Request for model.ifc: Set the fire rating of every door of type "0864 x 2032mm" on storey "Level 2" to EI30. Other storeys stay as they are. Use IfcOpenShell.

First a look at what the model holds.

```python
import ifcopenshell
import ifcopenshell.util.element

model = ifcopenshell.open("model.ifc")
print(model.schema)
storey = next(s for s in model.by_type("IfcBuildingStorey") if s.Name == "Level 2")
doors = [e for e in ifcopenshell.util.element.get_decomposition(storey) if e.is_a("IfcDoor")]
seen = {}
for e in doors:
    element_type = ifcopenshell.util.element.get_type(e)
    key = (element_type.Name if element_type != e and element_type else None, ifcopenshell.util.element.get_pset(e, "Pset_DoorCommon", "FireRating"))
    seen[key] = seen.get(key, 0) + 1
for (name, value), count in sorted(seen.items(), key=str):
    print(count, "x", name, "|", value)
```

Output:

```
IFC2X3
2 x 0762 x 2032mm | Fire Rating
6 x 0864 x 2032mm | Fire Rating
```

```python
import ifcopenshell
import ifcopenshell.api.pset
import ifcopenshell.util.element

model = ifcopenshell.open("model.ifc")

storey = next(s for s in model.by_type("IfcBuildingStorey") if s.Name == "Level 2")
doors = [e for e in ifcopenshell.util.element.get_decomposition(storey) if e.is_a("IfcDoor")]

count = 0
for e in doors:
    element_type = ifcopenshell.util.element.get_type(e)
    if element_type in (None, e) or element_type.Name != "0864 x 2032mm":
        continue
    # add_pset returns the element's existing set when there is one.
    pset = ifcopenshell.api.pset.add_pset(model, product=e, name="Pset_DoorCommon")
    ifcopenshell.api.pset.edit_pset(model, pset=pset, properties={"FireRating": "EI30"})
    count += 1

print(count, "doors updated")

model.write("model_edited.ifc")
```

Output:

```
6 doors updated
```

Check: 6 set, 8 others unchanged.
